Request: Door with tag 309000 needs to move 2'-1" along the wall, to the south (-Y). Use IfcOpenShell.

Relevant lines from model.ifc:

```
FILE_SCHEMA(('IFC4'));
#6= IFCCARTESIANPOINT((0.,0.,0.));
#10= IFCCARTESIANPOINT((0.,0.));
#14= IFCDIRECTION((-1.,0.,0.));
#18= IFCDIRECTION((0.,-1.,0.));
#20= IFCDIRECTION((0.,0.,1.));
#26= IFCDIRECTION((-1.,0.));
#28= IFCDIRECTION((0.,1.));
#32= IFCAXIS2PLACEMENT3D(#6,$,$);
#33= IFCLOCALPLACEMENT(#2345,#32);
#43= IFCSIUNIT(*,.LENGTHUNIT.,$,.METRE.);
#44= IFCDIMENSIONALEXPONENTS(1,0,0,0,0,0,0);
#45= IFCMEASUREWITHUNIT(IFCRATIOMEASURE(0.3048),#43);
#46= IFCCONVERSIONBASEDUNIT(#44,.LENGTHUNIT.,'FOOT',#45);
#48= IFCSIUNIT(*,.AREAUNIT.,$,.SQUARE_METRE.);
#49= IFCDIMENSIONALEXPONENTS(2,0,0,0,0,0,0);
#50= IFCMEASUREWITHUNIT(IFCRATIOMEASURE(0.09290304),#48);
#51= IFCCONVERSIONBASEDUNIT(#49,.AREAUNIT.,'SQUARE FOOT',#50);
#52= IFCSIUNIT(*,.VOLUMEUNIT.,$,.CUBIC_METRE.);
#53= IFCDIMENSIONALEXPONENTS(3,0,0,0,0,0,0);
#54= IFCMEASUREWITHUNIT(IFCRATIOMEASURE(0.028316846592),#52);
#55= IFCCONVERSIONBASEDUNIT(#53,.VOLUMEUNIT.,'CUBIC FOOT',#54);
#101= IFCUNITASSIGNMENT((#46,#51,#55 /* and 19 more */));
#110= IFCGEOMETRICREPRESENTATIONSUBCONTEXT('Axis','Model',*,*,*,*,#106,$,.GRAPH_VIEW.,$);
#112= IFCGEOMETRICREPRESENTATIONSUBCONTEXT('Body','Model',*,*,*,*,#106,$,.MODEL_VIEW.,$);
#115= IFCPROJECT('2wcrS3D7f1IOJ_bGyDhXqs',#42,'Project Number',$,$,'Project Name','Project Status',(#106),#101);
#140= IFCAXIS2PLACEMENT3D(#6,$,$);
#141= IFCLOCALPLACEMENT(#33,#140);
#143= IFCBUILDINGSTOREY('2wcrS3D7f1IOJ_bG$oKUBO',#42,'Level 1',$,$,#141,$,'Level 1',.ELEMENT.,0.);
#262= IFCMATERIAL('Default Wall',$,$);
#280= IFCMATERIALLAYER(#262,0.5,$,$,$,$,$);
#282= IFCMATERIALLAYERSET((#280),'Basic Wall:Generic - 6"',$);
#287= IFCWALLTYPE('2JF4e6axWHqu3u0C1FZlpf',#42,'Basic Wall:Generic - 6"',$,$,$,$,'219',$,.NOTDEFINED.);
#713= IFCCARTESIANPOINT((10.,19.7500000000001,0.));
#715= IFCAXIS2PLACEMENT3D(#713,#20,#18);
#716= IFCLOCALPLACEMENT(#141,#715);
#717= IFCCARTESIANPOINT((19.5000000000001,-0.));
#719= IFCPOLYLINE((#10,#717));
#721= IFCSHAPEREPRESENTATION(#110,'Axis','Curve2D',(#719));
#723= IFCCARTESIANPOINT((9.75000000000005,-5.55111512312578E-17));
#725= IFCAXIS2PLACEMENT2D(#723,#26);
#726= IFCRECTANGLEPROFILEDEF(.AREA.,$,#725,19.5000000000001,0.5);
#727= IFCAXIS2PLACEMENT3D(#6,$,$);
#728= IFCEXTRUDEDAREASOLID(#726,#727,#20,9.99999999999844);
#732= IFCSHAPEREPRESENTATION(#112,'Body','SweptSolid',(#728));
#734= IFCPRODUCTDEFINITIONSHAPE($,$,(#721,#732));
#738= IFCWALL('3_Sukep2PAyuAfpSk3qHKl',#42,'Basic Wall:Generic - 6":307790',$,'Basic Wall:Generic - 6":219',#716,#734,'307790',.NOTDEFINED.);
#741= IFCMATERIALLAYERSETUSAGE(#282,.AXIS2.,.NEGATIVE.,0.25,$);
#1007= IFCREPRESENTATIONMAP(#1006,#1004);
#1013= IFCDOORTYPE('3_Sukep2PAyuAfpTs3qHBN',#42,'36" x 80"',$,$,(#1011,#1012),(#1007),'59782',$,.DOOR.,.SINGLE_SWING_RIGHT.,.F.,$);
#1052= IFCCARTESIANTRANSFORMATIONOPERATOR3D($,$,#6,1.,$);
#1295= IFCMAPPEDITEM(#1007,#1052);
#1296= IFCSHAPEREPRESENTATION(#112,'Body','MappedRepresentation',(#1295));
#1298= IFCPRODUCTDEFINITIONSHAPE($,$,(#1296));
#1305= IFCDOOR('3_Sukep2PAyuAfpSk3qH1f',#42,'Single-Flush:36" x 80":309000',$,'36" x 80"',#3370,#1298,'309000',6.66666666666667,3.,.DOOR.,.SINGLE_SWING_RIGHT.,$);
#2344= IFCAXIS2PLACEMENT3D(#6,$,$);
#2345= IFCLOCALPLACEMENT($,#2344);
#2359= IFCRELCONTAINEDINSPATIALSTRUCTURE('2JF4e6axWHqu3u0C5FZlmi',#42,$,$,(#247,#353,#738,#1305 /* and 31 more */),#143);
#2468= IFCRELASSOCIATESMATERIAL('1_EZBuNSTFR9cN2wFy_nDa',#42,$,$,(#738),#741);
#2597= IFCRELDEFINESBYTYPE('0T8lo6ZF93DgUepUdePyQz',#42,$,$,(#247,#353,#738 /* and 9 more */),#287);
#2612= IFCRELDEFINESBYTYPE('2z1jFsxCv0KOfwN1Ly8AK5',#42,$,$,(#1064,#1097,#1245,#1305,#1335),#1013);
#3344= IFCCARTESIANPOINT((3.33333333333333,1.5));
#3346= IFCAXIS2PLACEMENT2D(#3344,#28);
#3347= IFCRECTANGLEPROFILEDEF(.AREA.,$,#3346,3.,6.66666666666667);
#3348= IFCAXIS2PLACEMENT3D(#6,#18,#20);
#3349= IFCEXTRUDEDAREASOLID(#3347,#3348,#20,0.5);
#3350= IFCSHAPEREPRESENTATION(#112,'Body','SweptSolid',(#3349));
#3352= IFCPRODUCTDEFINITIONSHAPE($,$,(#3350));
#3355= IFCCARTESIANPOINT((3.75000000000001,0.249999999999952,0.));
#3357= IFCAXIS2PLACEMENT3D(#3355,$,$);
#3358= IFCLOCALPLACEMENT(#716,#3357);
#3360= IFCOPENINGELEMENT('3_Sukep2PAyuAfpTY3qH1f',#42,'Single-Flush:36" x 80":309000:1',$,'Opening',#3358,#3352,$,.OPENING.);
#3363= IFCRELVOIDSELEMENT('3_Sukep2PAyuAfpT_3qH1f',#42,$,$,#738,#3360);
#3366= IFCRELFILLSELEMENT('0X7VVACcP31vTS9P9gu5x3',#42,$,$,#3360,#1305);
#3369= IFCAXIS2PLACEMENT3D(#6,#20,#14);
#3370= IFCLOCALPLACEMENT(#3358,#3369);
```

```python
import ifcopenshell
import ifcopenshell.api.geometry
import ifcopenshell.util.placement
import ifcopenshell.util.unit

model = ifcopenshell.open("model.ifc")
unit_scale = ifcopenshell.util.unit.calculate_unit_scale(model)

door = model.by_guid("3_Sukep2PAyuAfpSk3qH1f")
opening = door.FillsVoids[0].RelatingOpeningElement
wall = opening.VoidsElements[0].RelatingBuildingElement

wall_matrix = ifcopenshell.util.placement.get_local_placement(wall.ObjectPlacement)
shift = wall_matrix[:3, 0] * 25 * 0.0254 / unit_scale
before = ifcopenshell.util.placement.get_local_placement(door.ObjectPlacement)[:3, 3].copy()

# The door is placed relative to its opening, so it follows when the opening moves.
matrix = ifcopenshell.util.placement.get_local_placement(opening.ObjectPlacement)
matrix[:3, 3] += shift
ifcopenshell.api.geometry.edit_object_placement(
    model, product=opening, matrix=matrix, is_si=False, should_transform_children=True
)

after = ifcopenshell.util.placement.get_local_placement(door.ObjectPlacement)[:3, 3]
print("door moved by", (after - before).round(3) + 0.0)

model.write("model_rev.ifc")
```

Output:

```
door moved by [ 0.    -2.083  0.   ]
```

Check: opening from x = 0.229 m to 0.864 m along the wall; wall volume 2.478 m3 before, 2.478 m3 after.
